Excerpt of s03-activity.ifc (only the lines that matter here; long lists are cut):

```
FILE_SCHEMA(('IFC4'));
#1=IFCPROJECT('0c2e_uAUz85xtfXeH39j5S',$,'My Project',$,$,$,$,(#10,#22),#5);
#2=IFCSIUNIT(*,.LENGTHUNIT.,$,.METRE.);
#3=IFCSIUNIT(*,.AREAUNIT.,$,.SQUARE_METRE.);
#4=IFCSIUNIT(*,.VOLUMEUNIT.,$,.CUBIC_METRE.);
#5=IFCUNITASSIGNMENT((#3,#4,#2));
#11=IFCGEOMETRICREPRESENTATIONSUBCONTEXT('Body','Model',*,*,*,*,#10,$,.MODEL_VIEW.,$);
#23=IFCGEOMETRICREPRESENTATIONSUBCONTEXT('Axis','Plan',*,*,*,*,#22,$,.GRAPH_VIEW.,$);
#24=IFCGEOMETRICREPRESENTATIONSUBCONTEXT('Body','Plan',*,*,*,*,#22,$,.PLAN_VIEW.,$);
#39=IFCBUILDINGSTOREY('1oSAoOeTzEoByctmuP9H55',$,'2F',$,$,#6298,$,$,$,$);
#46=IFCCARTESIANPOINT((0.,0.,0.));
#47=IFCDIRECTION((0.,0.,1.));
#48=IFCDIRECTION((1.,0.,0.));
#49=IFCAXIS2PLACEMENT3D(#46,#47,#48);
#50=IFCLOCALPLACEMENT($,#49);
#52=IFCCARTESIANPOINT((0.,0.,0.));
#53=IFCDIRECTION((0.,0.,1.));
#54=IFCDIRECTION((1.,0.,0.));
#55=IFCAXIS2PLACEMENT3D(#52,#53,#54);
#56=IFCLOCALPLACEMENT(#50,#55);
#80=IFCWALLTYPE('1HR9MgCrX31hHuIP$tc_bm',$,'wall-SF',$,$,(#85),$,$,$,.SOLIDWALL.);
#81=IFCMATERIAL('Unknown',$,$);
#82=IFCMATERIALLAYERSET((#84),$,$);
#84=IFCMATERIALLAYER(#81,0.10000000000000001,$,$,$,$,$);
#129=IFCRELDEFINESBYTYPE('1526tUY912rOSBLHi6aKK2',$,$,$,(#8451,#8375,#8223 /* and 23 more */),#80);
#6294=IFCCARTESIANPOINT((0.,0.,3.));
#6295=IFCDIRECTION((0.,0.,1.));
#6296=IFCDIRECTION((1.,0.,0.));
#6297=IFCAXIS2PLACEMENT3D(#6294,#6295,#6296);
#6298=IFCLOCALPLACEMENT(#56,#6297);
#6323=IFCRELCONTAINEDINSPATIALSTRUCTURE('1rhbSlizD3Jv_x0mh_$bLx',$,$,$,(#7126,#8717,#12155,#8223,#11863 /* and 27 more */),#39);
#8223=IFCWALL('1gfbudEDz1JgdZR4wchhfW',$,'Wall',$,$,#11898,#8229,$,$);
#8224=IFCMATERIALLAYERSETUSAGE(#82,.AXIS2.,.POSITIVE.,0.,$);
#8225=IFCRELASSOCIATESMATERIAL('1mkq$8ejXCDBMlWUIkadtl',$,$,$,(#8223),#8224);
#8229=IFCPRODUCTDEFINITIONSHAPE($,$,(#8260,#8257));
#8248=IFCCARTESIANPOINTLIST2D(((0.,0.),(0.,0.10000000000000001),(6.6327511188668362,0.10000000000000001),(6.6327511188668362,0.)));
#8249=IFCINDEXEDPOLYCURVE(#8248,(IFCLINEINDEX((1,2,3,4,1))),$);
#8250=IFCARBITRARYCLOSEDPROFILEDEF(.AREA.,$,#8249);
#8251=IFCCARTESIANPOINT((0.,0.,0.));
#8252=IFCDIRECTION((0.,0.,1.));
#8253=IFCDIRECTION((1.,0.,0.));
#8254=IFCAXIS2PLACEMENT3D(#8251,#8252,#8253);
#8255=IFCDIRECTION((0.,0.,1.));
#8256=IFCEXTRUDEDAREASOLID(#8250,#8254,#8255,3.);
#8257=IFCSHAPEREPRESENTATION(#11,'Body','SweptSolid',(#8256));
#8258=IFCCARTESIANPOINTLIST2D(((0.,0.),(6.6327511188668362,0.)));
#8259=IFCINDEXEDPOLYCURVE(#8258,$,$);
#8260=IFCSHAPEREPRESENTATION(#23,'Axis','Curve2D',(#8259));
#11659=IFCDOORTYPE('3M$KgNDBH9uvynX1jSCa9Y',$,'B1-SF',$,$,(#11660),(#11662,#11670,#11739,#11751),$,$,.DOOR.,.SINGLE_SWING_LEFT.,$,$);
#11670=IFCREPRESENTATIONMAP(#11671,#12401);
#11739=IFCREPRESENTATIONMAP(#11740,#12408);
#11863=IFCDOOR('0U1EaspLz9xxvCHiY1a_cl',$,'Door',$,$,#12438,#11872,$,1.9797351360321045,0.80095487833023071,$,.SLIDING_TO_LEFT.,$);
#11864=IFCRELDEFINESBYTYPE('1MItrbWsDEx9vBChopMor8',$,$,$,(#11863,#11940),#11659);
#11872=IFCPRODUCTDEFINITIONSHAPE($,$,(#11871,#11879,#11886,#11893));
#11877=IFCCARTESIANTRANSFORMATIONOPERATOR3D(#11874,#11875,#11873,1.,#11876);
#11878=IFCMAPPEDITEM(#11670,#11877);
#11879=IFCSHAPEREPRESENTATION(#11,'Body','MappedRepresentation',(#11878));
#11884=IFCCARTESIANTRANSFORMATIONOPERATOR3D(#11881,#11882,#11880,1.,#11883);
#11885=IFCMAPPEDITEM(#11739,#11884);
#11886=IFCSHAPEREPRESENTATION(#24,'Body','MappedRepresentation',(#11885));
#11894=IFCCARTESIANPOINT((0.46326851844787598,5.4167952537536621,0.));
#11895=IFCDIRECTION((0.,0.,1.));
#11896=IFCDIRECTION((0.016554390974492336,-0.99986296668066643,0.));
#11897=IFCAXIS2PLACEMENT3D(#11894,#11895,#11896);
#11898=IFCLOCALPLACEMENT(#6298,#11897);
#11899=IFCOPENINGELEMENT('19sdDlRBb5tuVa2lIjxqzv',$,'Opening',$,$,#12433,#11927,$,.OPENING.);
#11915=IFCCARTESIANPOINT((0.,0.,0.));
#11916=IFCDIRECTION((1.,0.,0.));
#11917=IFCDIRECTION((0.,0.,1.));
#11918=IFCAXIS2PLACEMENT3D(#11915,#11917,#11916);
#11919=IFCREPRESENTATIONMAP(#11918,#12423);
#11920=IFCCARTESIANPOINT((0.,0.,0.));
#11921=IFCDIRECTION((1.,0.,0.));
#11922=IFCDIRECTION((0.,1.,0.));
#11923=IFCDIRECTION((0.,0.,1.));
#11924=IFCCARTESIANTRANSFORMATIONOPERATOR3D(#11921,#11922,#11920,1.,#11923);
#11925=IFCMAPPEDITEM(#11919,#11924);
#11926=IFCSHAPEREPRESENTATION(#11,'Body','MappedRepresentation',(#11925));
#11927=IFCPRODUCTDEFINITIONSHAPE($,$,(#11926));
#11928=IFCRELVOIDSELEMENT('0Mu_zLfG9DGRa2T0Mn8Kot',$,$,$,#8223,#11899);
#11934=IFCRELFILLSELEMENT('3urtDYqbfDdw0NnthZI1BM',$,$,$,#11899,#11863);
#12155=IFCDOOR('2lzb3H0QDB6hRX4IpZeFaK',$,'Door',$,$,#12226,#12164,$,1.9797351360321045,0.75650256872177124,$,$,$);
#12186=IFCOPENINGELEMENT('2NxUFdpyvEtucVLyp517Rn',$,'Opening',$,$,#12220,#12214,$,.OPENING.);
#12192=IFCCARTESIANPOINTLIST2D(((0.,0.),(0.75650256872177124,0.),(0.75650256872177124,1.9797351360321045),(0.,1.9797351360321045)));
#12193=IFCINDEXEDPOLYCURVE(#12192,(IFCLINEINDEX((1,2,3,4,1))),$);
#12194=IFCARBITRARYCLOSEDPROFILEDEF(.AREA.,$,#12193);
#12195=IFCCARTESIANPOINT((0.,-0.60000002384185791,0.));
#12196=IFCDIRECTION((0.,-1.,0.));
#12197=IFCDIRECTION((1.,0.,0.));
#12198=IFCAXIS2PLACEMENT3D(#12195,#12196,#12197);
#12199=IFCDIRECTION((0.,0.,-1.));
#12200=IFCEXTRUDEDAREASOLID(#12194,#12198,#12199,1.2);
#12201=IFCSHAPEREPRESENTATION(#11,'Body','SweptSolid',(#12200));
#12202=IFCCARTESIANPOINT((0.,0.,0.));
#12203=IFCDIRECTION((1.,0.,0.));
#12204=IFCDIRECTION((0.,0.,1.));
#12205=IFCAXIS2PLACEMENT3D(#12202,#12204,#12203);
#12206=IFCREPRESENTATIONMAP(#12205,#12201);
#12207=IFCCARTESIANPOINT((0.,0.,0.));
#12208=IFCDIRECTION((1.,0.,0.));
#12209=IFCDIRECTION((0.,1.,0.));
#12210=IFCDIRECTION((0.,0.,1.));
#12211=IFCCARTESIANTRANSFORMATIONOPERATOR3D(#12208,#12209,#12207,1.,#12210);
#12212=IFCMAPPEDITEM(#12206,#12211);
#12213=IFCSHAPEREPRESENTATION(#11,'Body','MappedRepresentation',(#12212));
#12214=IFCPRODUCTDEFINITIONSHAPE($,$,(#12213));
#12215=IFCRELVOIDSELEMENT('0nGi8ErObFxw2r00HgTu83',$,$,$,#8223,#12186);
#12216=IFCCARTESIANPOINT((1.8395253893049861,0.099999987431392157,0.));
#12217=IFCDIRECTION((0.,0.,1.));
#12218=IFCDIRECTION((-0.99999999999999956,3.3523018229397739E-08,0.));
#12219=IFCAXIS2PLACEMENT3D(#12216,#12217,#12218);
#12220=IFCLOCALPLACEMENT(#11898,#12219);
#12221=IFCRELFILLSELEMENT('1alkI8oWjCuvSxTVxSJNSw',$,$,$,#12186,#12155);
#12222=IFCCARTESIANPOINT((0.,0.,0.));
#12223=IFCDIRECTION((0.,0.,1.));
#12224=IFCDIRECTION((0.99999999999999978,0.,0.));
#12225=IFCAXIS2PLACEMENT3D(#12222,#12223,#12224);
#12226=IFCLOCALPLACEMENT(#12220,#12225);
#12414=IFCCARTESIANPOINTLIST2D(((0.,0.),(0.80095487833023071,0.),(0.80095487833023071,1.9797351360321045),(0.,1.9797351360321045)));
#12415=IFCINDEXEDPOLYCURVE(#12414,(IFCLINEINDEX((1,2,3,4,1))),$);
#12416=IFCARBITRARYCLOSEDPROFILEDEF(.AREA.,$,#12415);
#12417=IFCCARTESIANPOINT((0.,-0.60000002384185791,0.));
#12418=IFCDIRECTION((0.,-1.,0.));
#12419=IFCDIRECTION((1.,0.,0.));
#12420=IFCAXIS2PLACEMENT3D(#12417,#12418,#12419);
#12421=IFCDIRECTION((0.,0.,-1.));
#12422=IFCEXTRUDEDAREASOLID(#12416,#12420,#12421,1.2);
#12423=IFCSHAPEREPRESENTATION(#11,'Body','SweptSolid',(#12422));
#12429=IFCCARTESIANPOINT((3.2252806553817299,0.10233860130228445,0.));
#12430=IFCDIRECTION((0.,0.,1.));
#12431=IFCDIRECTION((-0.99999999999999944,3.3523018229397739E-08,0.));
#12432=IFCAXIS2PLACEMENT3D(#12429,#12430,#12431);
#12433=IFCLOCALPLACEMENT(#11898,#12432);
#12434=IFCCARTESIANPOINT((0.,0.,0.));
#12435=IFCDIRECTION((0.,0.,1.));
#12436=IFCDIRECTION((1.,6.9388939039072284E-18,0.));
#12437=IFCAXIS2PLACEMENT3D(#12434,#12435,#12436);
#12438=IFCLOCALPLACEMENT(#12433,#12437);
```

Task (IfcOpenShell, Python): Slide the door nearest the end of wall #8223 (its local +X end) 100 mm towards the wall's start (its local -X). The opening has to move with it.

```python
import ifcopenshell
import ifcopenshell.api.geometry
import ifcopenshell.util.placement
import ifcopenshell.util.unit

model = ifcopenshell.open("s03-activity.ifc")
unit_scale = ifcopenshell.util.unit.calculate_unit_scale(model)

door = model.by_guid("0U1EaspLz9xxvCHiY1a_cl")
opening = door.FillsVoids[0].RelatingOpeningElement
wall = opening.VoidsElements[0].RelatingBuildingElement

wall_matrix = ifcopenshell.util.placement.get_local_placement(wall.ObjectPlacement)
shift = wall_matrix[:3, 0] * -0.1 / unit_scale
before = ifcopenshell.util.placement.get_local_placement(door.ObjectPlacement)[:3, 3].copy()

# The door is placed relative to its opening, so it follows when the opening moves.
matrix = ifcopenshell.util.placement.get_local_placement(opening.ObjectPlacement)
matrix[:3, 3] += shift
ifcopenshell.api.geometry.edit_object_placement(
    model, product=opening, matrix=matrix, is_si=False, should_transform_children=True
)

after = ifcopenshell.util.placement.get_local_placement(door.ObjectPlacement)[:3, 3]
print("door moved by", (after - before).round(3) + 0.0)

model.write("s03-activity_rev.ifc")
```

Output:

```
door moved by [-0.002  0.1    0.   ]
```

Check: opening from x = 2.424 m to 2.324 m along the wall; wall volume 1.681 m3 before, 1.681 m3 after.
